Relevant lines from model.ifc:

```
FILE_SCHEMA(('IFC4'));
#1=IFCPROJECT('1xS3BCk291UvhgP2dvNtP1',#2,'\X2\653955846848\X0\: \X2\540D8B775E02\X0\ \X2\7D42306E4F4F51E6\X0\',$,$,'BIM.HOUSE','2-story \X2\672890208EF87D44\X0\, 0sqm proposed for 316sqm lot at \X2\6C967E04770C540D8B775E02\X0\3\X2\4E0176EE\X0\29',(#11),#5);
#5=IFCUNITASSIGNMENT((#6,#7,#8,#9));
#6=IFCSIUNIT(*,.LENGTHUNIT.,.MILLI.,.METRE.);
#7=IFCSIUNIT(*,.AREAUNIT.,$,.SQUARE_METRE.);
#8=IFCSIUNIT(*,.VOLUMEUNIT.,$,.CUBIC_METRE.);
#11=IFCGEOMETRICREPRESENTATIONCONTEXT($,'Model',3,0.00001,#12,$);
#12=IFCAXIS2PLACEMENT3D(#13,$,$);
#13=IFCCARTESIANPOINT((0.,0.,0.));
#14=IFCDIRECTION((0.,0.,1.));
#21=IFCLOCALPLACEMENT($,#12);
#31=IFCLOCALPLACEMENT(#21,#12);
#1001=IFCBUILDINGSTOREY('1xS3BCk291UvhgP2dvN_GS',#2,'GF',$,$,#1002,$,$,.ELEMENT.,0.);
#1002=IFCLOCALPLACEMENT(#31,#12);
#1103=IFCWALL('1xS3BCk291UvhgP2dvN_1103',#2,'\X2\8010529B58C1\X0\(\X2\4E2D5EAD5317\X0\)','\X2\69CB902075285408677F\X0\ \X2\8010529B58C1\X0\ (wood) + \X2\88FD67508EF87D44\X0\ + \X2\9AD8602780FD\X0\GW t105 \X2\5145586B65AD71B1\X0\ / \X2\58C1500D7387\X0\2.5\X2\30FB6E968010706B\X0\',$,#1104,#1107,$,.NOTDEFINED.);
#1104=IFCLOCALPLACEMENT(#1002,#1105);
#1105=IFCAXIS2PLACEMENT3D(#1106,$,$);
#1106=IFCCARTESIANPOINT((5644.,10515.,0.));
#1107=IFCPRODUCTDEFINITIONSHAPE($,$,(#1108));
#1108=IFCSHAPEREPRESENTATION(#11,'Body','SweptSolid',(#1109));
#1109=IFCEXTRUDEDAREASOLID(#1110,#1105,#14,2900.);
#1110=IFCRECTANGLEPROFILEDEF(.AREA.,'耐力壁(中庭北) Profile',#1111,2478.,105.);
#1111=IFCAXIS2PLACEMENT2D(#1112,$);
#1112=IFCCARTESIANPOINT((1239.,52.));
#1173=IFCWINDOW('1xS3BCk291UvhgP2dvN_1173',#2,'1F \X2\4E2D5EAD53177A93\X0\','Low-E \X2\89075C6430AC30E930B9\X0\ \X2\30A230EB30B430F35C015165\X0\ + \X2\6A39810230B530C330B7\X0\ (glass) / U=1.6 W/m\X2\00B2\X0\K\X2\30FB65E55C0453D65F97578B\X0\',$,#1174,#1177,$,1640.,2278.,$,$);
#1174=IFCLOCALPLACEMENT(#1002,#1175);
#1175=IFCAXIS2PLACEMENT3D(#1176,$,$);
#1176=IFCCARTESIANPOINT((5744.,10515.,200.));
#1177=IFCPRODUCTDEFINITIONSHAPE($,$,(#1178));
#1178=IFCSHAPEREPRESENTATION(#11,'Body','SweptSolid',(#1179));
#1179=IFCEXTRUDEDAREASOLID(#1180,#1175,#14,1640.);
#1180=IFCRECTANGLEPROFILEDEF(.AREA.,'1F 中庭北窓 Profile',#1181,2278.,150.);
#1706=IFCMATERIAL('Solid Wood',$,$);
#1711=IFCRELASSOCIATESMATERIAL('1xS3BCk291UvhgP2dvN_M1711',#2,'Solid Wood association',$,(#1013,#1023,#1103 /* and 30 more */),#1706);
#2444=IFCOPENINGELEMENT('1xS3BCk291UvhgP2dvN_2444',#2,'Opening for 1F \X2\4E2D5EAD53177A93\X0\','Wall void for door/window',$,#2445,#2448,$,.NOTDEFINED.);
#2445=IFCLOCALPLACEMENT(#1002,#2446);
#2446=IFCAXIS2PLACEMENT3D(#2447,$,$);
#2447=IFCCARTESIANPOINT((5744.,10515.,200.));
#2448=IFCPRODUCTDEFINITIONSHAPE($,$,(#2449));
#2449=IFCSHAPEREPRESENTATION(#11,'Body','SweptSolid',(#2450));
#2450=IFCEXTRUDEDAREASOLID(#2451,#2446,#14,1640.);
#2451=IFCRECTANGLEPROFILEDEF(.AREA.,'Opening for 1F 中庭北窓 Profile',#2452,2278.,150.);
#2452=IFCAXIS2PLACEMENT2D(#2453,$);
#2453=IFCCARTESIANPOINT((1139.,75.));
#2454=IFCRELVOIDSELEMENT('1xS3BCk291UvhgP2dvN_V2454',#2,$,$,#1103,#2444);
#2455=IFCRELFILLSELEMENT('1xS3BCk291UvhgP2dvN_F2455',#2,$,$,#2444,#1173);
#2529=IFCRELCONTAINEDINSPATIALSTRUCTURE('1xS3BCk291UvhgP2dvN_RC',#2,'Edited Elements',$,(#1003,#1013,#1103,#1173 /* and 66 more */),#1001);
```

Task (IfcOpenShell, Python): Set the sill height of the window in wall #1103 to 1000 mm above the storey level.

```python
import numpy as np
import ifcopenshell
import ifcopenshell.api.geometry
import ifcopenshell.geom
import ifcopenshell.util.element
import ifcopenshell.util.placement
import ifcopenshell.util.shape
import ifcopenshell.util.unit

model = ifcopenshell.open("model.ifc")
unit_scale = ifcopenshell.util.unit.calculate_unit_scale(model)

window = model.by_guid("1xS3BCk291UvhgP2dvN_1173")
opening = window.FillsVoids[0].RelatingOpeningElement
storey = ifcopenshell.util.element.get_container(window, ifc_class="IfcBuildingStorey")
level = ifcopenshell.util.placement.get_local_placement(storey.ObjectPlacement)[2, 3]

# The opening's origin need not be at the sill, so measure its lowest point.
shape = ifcopenshell.geom.create_shape(ifcopenshell.geom.settings(), opening)
bottom = ifcopenshell.util.shape.get_shape_bottom_elevation(shape, shape.geometry) / unit_scale
dz = level + 1 / unit_scale - bottom

shift = np.array([0.0, 0.0, dz])
# The window is not placed relative to its opening, so move both.
for product in (opening, window):
    matrix = ifcopenshell.util.placement.get_local_placement(product.ObjectPlacement)
    matrix[:3, 3] += shift
    ifcopenshell.api.geometry.edit_object_placement(model, product=product, matrix=matrix, is_si=False)

print(f"moved by {dz * unit_scale:+.3f} m")

model.write("model_v2.ifc")
```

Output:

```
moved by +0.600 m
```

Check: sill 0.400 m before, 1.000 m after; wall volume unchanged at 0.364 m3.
